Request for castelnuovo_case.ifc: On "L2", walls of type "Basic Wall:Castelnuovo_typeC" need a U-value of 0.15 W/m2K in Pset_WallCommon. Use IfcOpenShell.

First a look at what the model holds.

```python
import ifcopenshell
import ifcopenshell.util.element

model = ifcopenshell.open("castelnuovo_case.ifc")
print(model.schema)
storey = next(s for s in model.by_type("IfcBuildingStorey") if s.Name == "L2")
walls = [e for e in ifcopenshell.util.element.get_decomposition(storey) if e.is_a("IfcWall")]
seen = {}
for e in walls:
    element_type = ifcopenshell.util.element.get_type(e)
    key = (element_type.Name if element_type != e and element_type else None, ifcopenshell.util.element.get_pset(e, "Pset_WallCommon", "ThermalTransmittance"))
    seen[key] = seen.get(key, 0) + 1
for (name, value), count in sorted(seen.items(), key=str):
    print(count, "x", name, "|", value)
```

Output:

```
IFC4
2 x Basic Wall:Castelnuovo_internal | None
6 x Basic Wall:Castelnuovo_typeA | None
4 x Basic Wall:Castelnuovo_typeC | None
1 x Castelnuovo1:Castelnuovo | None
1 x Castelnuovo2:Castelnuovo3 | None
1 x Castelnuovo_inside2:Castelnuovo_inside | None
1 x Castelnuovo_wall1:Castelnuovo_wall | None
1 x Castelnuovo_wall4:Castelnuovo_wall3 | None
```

```python
import ifcopenshell
import ifcopenshell.api.pset
import ifcopenshell.util.element

model = ifcopenshell.open("castelnuovo_case.ifc")

storey = next(s for s in model.by_type("IfcBuildingStorey") if s.Name == "L2")
walls = [e for e in ifcopenshell.util.element.get_decomposition(storey) if e.is_a("IfcWall")]

count = 0
for e in walls:
    element_type = ifcopenshell.util.element.get_type(e)
    if element_type in (None, e) or element_type.Name != "Basic Wall:Castelnuovo_typeC":
        continue
    # add_pset returns the element's existing set when there is one.
    pset = ifcopenshell.api.pset.add_pset(model, product=e, name="Pset_WallCommon")
    ifcopenshell.api.pset.edit_pset(model, pset=pset, properties={"ThermalTransmittance": 0.15})
    count += 1

print(count, "walls updated")

model.write("castelnuovo_case_v2.ifc")
```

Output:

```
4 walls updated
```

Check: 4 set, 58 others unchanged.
